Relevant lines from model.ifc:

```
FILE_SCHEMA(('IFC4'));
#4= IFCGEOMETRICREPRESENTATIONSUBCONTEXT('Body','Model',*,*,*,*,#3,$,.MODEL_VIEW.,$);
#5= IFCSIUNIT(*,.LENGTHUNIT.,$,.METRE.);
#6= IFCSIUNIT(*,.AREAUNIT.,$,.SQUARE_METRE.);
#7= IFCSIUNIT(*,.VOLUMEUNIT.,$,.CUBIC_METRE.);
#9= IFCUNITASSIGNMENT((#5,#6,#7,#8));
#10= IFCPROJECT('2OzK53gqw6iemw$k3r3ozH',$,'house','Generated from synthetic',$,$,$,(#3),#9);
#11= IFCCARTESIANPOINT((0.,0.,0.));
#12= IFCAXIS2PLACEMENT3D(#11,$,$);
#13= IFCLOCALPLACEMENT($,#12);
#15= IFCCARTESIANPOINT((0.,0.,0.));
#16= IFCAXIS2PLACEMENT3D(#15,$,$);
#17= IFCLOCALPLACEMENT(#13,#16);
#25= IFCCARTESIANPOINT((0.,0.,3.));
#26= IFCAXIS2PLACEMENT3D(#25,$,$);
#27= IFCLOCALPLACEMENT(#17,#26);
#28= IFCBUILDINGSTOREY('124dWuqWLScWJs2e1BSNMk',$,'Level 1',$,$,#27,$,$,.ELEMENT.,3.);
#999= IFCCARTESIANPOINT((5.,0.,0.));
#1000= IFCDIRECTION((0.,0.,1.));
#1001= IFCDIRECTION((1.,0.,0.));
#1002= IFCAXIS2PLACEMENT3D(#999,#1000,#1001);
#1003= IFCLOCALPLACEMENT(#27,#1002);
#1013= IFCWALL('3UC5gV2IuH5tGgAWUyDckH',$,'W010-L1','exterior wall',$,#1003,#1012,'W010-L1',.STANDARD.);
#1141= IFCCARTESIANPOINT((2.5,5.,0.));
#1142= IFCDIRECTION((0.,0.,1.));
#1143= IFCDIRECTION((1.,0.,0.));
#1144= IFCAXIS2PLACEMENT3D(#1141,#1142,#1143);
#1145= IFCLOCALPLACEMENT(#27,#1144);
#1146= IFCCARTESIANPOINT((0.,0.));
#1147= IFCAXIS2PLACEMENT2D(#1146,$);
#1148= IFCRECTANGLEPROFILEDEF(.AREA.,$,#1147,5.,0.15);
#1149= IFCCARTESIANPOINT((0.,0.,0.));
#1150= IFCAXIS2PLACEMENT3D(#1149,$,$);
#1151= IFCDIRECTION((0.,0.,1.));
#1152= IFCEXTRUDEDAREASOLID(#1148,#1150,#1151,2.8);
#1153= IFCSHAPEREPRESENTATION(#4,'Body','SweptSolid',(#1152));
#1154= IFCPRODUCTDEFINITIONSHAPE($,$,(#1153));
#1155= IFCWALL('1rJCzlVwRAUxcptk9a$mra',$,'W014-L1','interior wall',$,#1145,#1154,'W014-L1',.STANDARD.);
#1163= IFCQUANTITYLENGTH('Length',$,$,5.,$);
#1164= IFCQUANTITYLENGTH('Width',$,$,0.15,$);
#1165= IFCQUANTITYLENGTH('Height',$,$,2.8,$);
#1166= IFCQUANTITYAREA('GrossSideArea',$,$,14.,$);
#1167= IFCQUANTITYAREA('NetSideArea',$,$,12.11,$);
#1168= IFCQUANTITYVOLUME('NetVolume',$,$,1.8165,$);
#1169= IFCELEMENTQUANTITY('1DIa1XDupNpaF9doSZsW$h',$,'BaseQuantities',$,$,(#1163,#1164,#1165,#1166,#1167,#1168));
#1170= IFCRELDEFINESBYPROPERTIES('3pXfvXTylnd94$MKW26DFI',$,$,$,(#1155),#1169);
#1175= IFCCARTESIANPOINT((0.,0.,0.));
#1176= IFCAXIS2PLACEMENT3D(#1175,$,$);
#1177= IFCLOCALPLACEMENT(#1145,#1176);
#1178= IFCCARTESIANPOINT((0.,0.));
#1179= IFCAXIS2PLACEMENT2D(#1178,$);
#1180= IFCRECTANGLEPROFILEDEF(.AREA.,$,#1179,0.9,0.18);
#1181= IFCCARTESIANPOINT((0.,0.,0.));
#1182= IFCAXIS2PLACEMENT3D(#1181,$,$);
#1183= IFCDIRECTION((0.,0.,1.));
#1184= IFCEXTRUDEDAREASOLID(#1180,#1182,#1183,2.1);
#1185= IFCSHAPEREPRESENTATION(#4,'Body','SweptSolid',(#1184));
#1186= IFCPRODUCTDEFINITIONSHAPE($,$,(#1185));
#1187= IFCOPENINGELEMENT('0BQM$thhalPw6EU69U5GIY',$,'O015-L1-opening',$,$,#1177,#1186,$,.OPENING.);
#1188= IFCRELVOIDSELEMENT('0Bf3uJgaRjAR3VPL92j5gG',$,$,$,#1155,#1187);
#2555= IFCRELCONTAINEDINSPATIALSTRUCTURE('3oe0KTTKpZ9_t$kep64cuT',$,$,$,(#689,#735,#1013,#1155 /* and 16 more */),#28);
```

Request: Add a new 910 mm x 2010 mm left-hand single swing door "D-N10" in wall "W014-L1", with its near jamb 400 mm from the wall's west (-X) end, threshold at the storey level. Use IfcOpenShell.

```python
import numpy as np
import ifcopenshell
import ifcopenshell.api.feature
import ifcopenshell.api.geometry
import ifcopenshell.api.pset
import ifcopenshell.api.root
import ifcopenshell.api.spatial
import ifcopenshell.geom
import ifcopenshell.util.element
import ifcopenshell.util.placement
import ifcopenshell.util.representation
import ifcopenshell.util.shape
import ifcopenshell.util.unit

model = ifcopenshell.open("model.ifc")
unit_scale = ifcopenshell.util.unit.calculate_unit_scale(model)
area_scale = ifcopenshell.util.unit.calculate_unit_scale(model, "AREAUNIT")
volume_scale = ifcopenshell.util.unit.calculate_unit_scale(model, "VOLUMEUNIT")
settings = ifcopenshell.geom.settings()


def volume(element):
    """Net volume in cubic metres, openings subtracted."""
    shape = ifcopenshell.geom.create_shape(settings, element)
    return ifcopenshell.util.shape.get_volume(shape.geometry)


wall = model.by_guid("1rJCzlVwRAUxcptk9a$mra")
storey = ifcopenshell.util.element.get_container(wall, ifc_class="IfcBuildingStorey")
context = ifcopenshell.util.representation.get_context(model, "Model", "Body", "MODEL_VIEW")
before = volume(wall)

width, height, from_end, sill = 0.91, 2.01, 0.4, 0.0  # metres

# The wall runs along its own X axis, and the end named is its -X end.
wall_shape = ifcopenshell.geom.create_shape(settings, wall)
x, y, z = ifcopenshell.util.shape.get_vertices(wall_shape.geometry).T
start = x.min() + from_end
face, thickness = float(y.min()), float(y.max() - y.min())
wall_matrix = ifcopenshell.util.placement.get_local_placement(wall.ObjectPlacement)
level = ifcopenshell.util.placement.get_local_placement(storey.ObjectPlacement)[2, 3]


def in_wall(x, y):
    """Placement at x, y metres in the wall's axes, at sill height."""
    matrix = wall_matrix.copy()
    matrix[:, 3] = wall_matrix @ np.array([x / unit_scale, y / unit_scale, 0.0, 1.0])
    matrix[2, 3] = level + sill / unit_scale
    return matrix


# Opening: a box that overshoots both wall faces by 50 mm.
opening = ifcopenshell.api.root.create_entity(model, ifc_class="IfcOpeningElement", predefined_type="OPENING")
box = ifcopenshell.api.geometry.add_wall_representation(
    model, context=context, length=width, height=height, thickness=thickness + 0.1
)
ifcopenshell.api.geometry.assign_representation(model, product=opening, representation=box)
ifcopenshell.api.geometry.edit_object_placement(model, product=opening, matrix=in_wall(start, face - 0.05), is_si=False)
ifcopenshell.api.feature.add_feature(model, feature=opening, element=wall)

door = ifcopenshell.api.root.create_entity(model, ifc_class="IfcDoor", name="D-N10", predefined_type="DOOR")
door.OverallWidth, door.OverallHeight = width / unit_scale, height / unit_scale
door.OperationType = "SINGLE_SWING_LEFT"
body = ifcopenshell.api.geometry.add_door_representation(
    model,
    context=context,
    overall_width=door.OverallWidth,
    overall_height=door.OverallHeight,
    operation_type="SINGLE_SWING_LEFT",
    lining_properties={"LiningDepth": thickness / unit_scale, "ThresholdDepth": thickness / unit_scale},
)
ifcopenshell.api.geometry.assign_representation(model, product=door, representation=body)
ifcopenshell.api.spatial.assign_container(model, products=[door], relating_structure=storey)
ifcopenshell.api.feature.add_filling(model, opening=opening, element=door)

# The lining spans the wall, so the door starts at the wall face.
ifcopenshell.api.geometry.edit_object_placement(model, product=door, matrix=in_wall(start, face), is_si=False)

after = volume(wall)

# Update the wall's stored quantities.
qto = model.by_id(ifcopenshell.util.element.get_pset(wall, "BaseQuantities", should_inherit=False)["id"])
ifcopenshell.api.pset.edit_qto(model, qto=qto, properties={
    "NetSideArea": after / thickness / area_scale,
    "NetVolume": after / volume_scale,
})

print(f"wall volume {before:.3f} -> {after:.3f} m3")

model.write("model-out.ifc")
```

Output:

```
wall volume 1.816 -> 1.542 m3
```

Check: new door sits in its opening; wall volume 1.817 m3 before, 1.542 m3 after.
